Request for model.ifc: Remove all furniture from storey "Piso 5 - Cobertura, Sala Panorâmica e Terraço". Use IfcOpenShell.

First a look at what the model holds.

```python
import ifcopenshell
import ifcopenshell.util.element

model = ifcopenshell.open("model.ifc")
print(model.schema)
storey = next(s for s in model.by_type("IfcBuildingStorey") if s.Name == "Piso 5 - Cobertura, Sala Panorâmica e Terraço")
furniture = [e for e in ifcopenshell.util.element.get_decomposition(storey) if e.is_a("IfcFurnishingElement")]
seen = {}
for e in furniture:
    element_type = ifcopenshell.util.element.get_type(e)
    name = element_type.Name if element_type not in (None, e) else None
    seen[name] = seen.get(name, 0) + 1
for name, count in sorted(seen.items(), key=str):
    print(count, "x", name)
```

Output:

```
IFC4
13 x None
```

```python
import ifcopenshell
import ifcopenshell.api.root
import ifcopenshell.util.element

model = ifcopenshell.open("model.ifc")

storey = next(s for s in model.by_type("IfcBuildingStorey") if s.Name == "Piso 5 - Cobertura, Sala Panorâmica e Terraço")
furniture = [e for e in ifcopenshell.util.element.get_decomposition(storey) if e.is_a("IfcFurnishingElement")]

for e in furniture:
    ifcopenshell.api.root.remove_product(model, product=e)
print(len(furniture), "removed")

model.write("model_v2.ifc")
```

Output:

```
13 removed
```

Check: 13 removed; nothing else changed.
